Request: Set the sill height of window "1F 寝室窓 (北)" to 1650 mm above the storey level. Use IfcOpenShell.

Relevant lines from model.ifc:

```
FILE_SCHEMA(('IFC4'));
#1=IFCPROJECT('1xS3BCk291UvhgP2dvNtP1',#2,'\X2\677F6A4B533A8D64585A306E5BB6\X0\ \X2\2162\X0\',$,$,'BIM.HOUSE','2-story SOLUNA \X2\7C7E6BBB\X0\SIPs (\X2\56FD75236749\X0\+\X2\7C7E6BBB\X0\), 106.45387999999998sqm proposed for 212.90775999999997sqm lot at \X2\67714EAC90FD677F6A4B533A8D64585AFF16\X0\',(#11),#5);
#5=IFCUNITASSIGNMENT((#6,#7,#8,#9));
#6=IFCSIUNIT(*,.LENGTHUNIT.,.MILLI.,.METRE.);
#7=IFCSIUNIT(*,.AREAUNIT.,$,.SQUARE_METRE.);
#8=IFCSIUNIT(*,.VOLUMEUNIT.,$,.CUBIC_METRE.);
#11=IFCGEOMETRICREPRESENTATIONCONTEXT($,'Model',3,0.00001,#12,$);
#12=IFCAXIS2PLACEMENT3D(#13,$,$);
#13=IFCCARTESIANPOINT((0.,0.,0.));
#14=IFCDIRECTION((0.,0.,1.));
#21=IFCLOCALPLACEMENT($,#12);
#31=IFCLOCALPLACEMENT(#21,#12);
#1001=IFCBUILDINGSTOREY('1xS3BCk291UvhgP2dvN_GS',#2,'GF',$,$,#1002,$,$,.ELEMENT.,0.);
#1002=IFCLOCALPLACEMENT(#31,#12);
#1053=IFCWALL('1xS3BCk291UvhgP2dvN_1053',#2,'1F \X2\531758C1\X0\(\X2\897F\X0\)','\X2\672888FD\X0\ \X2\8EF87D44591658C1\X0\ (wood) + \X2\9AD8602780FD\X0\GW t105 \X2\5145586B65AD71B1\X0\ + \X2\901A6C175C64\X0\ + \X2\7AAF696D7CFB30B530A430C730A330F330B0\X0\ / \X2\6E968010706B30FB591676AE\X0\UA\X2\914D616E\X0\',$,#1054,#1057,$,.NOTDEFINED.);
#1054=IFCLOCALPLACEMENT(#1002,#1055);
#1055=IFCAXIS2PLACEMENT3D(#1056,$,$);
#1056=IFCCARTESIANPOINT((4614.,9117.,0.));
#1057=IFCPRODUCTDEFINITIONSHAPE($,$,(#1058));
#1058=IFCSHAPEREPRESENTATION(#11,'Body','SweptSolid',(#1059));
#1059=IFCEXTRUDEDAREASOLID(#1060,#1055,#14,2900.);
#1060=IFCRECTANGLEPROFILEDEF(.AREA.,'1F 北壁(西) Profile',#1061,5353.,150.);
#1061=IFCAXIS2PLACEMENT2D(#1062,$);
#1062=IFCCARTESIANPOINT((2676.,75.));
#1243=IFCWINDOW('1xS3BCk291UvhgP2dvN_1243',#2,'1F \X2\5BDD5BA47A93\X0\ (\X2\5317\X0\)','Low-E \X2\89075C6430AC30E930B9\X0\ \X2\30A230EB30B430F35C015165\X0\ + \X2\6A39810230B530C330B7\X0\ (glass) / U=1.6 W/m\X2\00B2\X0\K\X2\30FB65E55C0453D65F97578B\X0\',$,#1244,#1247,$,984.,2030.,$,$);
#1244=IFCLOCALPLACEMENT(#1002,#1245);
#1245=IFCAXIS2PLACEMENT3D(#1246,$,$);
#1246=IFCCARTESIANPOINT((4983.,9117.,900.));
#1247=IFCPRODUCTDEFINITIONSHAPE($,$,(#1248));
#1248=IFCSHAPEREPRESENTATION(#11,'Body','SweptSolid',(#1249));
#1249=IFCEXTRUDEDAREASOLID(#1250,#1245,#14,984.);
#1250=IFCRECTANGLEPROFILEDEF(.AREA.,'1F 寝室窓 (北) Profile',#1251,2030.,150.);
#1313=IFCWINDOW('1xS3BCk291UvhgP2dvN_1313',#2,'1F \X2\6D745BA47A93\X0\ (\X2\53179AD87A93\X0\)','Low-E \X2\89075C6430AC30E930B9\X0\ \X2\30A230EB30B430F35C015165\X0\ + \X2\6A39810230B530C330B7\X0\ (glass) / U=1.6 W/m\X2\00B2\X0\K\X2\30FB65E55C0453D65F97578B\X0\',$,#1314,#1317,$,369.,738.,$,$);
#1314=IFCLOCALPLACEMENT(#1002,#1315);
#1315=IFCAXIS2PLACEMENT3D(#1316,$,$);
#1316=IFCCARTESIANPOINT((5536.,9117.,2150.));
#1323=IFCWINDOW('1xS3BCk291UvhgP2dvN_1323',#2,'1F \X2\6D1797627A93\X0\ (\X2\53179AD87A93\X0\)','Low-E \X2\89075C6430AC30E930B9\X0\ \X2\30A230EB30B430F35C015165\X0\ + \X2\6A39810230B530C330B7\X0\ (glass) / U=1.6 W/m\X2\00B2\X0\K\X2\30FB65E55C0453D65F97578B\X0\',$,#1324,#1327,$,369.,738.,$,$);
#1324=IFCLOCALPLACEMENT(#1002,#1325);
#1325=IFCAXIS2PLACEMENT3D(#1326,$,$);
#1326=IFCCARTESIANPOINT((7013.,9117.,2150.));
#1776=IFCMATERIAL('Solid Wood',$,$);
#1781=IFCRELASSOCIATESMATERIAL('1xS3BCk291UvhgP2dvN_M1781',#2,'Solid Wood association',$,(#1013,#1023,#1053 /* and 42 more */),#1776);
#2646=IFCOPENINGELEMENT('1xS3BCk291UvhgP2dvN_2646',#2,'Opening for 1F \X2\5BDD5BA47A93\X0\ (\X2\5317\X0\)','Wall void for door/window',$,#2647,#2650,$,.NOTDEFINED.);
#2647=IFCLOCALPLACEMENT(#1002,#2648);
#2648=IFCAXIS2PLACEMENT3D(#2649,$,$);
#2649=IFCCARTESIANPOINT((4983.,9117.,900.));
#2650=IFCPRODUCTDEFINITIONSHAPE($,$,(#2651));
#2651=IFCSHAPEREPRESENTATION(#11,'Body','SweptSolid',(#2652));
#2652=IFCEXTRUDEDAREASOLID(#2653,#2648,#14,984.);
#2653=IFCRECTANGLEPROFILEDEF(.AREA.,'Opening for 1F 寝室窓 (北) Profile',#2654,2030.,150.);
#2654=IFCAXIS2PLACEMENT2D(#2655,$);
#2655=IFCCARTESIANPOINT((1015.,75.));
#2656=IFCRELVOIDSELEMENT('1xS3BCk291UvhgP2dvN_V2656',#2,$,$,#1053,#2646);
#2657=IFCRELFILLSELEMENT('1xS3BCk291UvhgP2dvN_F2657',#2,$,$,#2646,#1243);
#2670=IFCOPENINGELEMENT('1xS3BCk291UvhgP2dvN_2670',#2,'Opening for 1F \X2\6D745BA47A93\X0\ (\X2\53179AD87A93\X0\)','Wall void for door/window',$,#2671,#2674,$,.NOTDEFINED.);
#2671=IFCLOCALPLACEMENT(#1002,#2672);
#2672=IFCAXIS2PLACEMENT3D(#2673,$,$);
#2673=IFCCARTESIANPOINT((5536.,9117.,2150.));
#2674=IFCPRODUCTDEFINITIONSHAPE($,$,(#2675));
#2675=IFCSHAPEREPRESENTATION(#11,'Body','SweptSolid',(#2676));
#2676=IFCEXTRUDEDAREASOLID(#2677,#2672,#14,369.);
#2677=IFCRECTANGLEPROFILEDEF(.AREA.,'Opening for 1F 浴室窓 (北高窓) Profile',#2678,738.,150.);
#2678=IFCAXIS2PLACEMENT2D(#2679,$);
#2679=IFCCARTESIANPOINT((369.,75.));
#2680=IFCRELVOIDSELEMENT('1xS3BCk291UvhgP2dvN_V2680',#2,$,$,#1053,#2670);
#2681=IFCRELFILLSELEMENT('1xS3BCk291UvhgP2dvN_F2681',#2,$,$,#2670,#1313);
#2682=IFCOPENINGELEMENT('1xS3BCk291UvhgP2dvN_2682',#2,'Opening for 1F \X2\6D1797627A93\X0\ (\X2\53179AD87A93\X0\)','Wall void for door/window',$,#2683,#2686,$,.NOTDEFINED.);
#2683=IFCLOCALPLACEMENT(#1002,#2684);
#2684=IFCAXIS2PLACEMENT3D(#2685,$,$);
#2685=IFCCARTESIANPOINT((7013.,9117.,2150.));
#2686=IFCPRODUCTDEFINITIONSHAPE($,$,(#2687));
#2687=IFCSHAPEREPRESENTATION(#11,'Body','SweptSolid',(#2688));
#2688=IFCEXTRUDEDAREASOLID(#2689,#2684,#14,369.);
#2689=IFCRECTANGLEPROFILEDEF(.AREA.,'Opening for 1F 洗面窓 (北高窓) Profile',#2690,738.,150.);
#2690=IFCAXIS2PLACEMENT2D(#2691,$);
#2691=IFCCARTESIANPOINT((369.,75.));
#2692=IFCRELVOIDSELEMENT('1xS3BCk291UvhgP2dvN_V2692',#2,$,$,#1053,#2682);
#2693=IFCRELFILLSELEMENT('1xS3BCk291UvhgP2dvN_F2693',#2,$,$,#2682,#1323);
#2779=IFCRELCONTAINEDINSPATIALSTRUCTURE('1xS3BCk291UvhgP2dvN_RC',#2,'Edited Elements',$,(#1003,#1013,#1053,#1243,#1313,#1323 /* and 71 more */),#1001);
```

```python
import numpy as np
import ifcopenshell
import ifcopenshell.api.geometry
import ifcopenshell.geom
import ifcopenshell.util.element
import ifcopenshell.util.placement
import ifcopenshell.util.shape
import ifcopenshell.util.unit

model = ifcopenshell.open("model.ifc")
unit_scale = ifcopenshell.util.unit.calculate_unit_scale(model)

window = model.by_guid("1xS3BCk291UvhgP2dvN_1243")
opening = window.FillsVoids[0].RelatingOpeningElement
storey = ifcopenshell.util.element.get_container(window, ifc_class="IfcBuildingStorey")
level = ifcopenshell.util.placement.get_local_placement(storey.ObjectPlacement)[2, 3]

# The opening's origin need not be at the sill, so measure its lowest point.
shape = ifcopenshell.geom.create_shape(ifcopenshell.geom.settings(), opening)
bottom = ifcopenshell.util.shape.get_shape_bottom_elevation(shape, shape.geometry) / unit_scale
dz = level + 1650.0 - bottom

shift = np.array([0.0, 0.0, dz])
# The window is not placed relative to its opening, so move both.
for product in (opening, window):
    matrix = ifcopenshell.util.placement.get_local_placement(product.ObjectPlacement)
    matrix[:3, 3] += shift
    ifcopenshell.api.geometry.edit_object_placement(model, product=product, matrix=matrix, is_si=False)

print(f"moved by {dz * unit_scale:+.3f} m")

model.write("model_updated.ifc")
```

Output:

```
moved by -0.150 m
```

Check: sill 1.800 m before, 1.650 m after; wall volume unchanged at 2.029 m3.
